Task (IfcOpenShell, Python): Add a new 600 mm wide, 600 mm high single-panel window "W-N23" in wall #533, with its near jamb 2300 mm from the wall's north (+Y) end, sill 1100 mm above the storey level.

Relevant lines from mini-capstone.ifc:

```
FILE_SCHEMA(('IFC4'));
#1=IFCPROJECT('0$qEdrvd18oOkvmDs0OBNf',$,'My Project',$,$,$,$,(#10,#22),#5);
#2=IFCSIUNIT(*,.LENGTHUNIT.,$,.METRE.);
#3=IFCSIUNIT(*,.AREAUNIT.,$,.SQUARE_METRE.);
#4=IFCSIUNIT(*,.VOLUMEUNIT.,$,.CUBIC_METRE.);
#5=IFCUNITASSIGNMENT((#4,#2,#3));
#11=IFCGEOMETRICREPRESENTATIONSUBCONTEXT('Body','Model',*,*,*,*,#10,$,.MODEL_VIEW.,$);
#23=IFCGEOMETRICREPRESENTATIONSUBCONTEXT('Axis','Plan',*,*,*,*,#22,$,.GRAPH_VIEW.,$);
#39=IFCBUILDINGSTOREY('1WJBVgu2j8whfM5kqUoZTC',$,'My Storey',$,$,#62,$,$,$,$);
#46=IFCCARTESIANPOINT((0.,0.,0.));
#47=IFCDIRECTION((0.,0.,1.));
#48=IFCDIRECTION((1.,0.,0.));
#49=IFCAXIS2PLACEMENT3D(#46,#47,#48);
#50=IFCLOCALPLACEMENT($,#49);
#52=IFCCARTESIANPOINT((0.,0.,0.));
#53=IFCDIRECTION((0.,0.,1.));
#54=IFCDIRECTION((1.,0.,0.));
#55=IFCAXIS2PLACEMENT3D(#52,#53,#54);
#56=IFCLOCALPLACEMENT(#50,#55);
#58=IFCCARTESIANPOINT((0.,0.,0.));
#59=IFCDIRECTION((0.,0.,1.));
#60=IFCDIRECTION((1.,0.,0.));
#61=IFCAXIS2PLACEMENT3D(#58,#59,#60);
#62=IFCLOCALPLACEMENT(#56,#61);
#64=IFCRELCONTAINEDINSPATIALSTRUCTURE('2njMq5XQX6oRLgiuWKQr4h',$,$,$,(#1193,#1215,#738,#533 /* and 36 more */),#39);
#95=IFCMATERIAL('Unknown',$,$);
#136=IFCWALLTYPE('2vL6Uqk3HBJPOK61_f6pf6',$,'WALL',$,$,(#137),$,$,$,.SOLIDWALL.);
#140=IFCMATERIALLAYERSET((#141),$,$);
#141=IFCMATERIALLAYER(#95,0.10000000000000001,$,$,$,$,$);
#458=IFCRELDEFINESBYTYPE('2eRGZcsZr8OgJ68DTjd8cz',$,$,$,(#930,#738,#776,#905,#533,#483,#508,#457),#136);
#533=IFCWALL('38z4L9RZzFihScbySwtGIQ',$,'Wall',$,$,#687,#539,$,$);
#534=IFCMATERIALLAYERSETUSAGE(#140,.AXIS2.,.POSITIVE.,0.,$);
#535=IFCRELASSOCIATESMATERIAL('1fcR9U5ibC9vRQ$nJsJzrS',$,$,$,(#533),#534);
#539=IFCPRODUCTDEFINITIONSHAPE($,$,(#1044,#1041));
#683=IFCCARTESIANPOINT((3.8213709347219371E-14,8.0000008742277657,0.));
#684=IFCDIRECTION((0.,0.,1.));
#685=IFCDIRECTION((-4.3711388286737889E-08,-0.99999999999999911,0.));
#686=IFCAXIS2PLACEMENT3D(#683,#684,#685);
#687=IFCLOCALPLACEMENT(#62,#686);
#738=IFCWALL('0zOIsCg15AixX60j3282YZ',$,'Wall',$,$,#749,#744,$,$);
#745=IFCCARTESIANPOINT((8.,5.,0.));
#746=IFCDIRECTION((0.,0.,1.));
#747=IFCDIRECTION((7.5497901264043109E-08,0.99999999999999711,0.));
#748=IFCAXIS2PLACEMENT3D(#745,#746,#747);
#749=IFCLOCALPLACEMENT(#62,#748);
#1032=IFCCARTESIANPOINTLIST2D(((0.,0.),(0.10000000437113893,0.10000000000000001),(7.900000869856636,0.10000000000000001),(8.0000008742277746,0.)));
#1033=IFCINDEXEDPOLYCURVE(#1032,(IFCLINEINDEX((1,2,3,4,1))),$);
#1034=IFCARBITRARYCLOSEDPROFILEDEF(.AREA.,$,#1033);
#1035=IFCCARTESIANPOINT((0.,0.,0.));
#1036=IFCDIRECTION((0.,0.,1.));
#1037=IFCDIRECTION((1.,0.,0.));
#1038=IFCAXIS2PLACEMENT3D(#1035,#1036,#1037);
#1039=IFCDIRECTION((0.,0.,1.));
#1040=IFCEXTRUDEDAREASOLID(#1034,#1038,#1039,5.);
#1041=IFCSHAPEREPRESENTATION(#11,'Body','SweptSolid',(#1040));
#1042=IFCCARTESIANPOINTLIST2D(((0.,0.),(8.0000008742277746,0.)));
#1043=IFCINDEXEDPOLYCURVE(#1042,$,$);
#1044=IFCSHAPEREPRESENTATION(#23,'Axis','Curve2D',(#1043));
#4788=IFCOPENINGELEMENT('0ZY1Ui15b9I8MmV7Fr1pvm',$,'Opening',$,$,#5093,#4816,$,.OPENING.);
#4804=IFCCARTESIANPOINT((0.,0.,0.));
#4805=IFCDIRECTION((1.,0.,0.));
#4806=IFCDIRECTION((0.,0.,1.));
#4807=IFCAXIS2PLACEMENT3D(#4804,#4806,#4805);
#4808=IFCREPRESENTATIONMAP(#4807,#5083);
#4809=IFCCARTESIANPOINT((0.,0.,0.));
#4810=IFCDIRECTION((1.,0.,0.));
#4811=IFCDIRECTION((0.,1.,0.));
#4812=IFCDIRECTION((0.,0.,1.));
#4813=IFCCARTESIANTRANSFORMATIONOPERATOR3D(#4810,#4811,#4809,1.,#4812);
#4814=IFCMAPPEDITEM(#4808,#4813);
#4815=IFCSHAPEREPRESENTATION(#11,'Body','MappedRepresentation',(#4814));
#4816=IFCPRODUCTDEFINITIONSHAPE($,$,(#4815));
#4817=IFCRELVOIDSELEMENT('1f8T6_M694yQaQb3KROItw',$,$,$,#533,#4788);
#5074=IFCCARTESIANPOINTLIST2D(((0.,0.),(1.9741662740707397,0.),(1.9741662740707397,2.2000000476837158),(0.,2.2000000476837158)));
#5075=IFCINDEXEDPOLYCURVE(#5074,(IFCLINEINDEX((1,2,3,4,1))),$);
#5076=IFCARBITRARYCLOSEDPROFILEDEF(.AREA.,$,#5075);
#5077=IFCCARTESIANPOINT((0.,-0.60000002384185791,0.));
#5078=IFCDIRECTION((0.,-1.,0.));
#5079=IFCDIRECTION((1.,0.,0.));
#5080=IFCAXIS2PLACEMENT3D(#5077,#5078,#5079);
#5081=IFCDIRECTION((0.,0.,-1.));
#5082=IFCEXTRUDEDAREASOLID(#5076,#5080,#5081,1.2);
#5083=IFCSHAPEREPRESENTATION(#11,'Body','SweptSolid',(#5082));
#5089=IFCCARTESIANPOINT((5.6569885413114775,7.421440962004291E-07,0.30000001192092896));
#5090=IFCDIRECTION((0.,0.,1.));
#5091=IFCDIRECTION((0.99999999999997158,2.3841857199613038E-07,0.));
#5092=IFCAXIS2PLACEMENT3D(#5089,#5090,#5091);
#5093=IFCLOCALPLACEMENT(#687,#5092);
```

```python
import numpy as np
import ifcopenshell
import ifcopenshell.api.feature
import ifcopenshell.api.geometry
import ifcopenshell.api.root
import ifcopenshell.api.spatial
import ifcopenshell.geom
import ifcopenshell.util.element
import ifcopenshell.util.placement
import ifcopenshell.util.representation
import ifcopenshell.util.shape
import ifcopenshell.util.unit

model = ifcopenshell.open("mini-capstone.ifc")
unit_scale = ifcopenshell.util.unit.calculate_unit_scale(model)
settings = ifcopenshell.geom.settings()


def volume(element):
    """Net volume in cubic metres, openings subtracted."""
    shape = ifcopenshell.geom.create_shape(settings, element)
    return ifcopenshell.util.shape.get_volume(shape.geometry)


wall = model.by_guid("38z4L9RZzFihScbySwtGIQ")
storey = ifcopenshell.util.element.get_container(wall, ifc_class="IfcBuildingStorey")
context = ifcopenshell.util.representation.get_context(model, "Model", "Body", "MODEL_VIEW")
before = volume(wall)

width, height, from_end, sill = 0.6, 0.6, 2.3, 1.1  # metres

# The wall runs along its own X axis, and the end named is its -X end.
wall_shape = ifcopenshell.geom.create_shape(settings, wall)
x, y, z = ifcopenshell.util.shape.get_vertices(wall_shape.geometry).T
start = x.min() + from_end
face, thickness = float(y.min()), float(y.max() - y.min())
wall_matrix = ifcopenshell.util.placement.get_local_placement(wall.ObjectPlacement)
level = ifcopenshell.util.placement.get_local_placement(storey.ObjectPlacement)[2, 3]


def in_wall(x, y):
    """Placement at x, y metres in the wall's axes, at sill height."""
    matrix = wall_matrix.copy()
    matrix[:, 3] = wall_matrix @ np.array([x / unit_scale, y / unit_scale, 0.0, 1.0])
    matrix[2, 3] = level + sill / unit_scale
    return matrix


# Opening: a box that overshoots both wall faces by 50 mm.
opening = ifcopenshell.api.root.create_entity(model, ifc_class="IfcOpeningElement", predefined_type="OPENING")
box = ifcopenshell.api.geometry.add_wall_representation(
    model, context=context, length=width, height=height, thickness=thickness + 0.1
)
ifcopenshell.api.geometry.assign_representation(model, product=opening, representation=box)
ifcopenshell.api.geometry.edit_object_placement(model, product=opening, matrix=in_wall(start, face - 0.05), is_si=False)
ifcopenshell.api.feature.add_feature(model, feature=opening, element=wall)

window = ifcopenshell.api.root.create_entity(model, ifc_class="IfcWindow", name="W-N23", predefined_type="WINDOW")
window.OverallWidth, window.OverallHeight = width / unit_scale, height / unit_scale
window.PartitioningType = "SINGLE_PANEL"
body = ifcopenshell.api.geometry.add_window_representation(
    model,
    context=context,
    overall_width=window.OverallWidth,
    overall_height=window.OverallHeight,
    partition_type="SINGLE_PANEL",
)
ifcopenshell.api.geometry.assign_representation(model, product=window, representation=body)
ifcopenshell.api.spatial.assign_container(model, products=[window], relating_structure=storey)
ifcopenshell.api.feature.add_filling(model, opening=opening, element=window)

# Centre the window in the wall's thickness.
ifcopenshell.api.geometry.edit_object_placement(model, product=window, matrix=in_wall(start, face), is_si=False)
window_shape = ifcopenshell.geom.create_shape(settings, window)
depth = ifcopenshell.util.shape.get_vertices(window_shape.geometry)[:, 1]
offset = face + thickness / 2 - (depth.min() + depth.max()) / 2
ifcopenshell.api.geometry.edit_object_placement(model, product=window, matrix=in_wall(start, offset), is_si=False)

after = volume(wall)

print(f"wall volume {before:.3f} -> {after:.3f} m3")

model.write("mini-capstone_edited.ifc")
```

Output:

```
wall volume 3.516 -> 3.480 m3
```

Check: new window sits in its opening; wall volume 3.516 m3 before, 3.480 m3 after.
